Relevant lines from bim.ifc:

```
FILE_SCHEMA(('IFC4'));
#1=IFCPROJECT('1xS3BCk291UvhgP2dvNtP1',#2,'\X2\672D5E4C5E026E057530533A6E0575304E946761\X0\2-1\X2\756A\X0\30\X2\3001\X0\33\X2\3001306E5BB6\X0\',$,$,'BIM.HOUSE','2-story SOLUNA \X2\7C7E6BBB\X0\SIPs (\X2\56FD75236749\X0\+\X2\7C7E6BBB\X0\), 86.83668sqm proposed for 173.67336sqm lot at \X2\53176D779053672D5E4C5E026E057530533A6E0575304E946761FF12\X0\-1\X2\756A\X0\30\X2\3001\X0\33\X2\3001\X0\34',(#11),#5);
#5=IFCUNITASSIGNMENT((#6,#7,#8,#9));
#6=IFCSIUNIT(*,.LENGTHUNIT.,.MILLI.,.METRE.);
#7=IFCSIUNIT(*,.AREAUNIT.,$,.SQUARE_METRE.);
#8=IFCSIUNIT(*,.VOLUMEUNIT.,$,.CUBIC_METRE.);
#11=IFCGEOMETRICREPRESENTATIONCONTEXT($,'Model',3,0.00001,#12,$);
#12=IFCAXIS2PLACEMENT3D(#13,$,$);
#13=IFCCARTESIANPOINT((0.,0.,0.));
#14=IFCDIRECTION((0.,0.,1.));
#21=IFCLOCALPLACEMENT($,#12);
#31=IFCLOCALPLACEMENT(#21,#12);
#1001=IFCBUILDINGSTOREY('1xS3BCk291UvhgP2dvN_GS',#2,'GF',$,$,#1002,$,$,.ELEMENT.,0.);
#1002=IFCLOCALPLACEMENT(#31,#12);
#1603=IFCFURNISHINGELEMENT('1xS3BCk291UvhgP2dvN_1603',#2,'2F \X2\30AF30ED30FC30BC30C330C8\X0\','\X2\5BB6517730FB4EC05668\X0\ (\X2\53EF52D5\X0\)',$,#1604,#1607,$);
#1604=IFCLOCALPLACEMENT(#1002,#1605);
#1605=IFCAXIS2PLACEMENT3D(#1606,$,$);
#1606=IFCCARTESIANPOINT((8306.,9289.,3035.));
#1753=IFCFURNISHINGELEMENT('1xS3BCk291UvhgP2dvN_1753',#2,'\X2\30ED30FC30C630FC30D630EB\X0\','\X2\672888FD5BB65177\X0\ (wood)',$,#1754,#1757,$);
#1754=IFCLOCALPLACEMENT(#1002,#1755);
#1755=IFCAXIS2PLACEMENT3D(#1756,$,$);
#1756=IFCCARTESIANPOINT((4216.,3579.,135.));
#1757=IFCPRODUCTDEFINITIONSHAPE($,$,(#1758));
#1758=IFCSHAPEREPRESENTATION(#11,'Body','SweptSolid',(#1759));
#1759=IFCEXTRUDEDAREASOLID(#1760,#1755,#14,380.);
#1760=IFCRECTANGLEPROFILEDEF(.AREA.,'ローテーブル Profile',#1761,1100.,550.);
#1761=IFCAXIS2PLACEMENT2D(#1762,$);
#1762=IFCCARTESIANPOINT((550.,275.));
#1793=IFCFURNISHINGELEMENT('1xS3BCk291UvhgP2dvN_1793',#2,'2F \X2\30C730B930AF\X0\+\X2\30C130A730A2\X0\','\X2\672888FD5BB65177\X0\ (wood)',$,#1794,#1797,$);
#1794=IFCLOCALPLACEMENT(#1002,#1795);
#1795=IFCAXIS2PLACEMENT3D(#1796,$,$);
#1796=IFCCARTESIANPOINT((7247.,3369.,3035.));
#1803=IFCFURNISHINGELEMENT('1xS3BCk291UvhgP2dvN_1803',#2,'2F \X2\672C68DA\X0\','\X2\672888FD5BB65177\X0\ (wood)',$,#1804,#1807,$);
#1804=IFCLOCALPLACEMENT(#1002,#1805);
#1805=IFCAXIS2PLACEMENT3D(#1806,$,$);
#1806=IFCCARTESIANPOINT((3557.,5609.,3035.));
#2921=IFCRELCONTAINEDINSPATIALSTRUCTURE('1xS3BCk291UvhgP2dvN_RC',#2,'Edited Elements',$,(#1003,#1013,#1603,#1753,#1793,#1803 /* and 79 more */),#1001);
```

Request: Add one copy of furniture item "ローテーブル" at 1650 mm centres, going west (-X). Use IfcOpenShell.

```python
import numpy as np
import ifcopenshell
import ifcopenshell.api.geometry
import ifcopenshell.api.root
import ifcopenshell.util.element
import ifcopenshell.util.placement

model = ifcopenshell.open("bim.ifc")


def reuse_history(source, copy):
    """copy_class also copies each property set's owner history, people and application; keep the originals."""
    for rel in copy.IsDefinedBy:
        if rel.is_a("IfcRelDefinesByProperties") and (history := rel.RelatingPropertyDefinition.OwnerHistory):
            rel.RelatingPropertyDefinition.OwnerHistory = source.OwnerHistory
            ifcopenshell.util.element.remove_deep2(model, history)


source = model.by_guid("1xS3BCk291UvhgP2dvN_1753")
base = ifcopenshell.util.placement.get_local_placement(source.ObjectPlacement)
step = np.array([-1.0, 0.0, 0.0]) * 1650.0

for i in range(1, 2):
    copy = ifcopenshell.api.root.copy_class(model, product=source)
    copy.Representation = ifcopenshell.util.element.copy_deep(
        model, source.Representation, exclude=["IfcGeometricRepresentationContext", "IfcRepresentationMap"]
    )
    reuse_history(source, copy)
    matrix = base.copy()
    matrix[:3, 3] += i * step
    print("added at", matrix[:3, 3].round(3) + 0.0)
    ifcopenshell.api.geometry.edit_object_placement(model, product=copy, matrix=matrix, is_si=False)

model.write("bim-out.ifc")
```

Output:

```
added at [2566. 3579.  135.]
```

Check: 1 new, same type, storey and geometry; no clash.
